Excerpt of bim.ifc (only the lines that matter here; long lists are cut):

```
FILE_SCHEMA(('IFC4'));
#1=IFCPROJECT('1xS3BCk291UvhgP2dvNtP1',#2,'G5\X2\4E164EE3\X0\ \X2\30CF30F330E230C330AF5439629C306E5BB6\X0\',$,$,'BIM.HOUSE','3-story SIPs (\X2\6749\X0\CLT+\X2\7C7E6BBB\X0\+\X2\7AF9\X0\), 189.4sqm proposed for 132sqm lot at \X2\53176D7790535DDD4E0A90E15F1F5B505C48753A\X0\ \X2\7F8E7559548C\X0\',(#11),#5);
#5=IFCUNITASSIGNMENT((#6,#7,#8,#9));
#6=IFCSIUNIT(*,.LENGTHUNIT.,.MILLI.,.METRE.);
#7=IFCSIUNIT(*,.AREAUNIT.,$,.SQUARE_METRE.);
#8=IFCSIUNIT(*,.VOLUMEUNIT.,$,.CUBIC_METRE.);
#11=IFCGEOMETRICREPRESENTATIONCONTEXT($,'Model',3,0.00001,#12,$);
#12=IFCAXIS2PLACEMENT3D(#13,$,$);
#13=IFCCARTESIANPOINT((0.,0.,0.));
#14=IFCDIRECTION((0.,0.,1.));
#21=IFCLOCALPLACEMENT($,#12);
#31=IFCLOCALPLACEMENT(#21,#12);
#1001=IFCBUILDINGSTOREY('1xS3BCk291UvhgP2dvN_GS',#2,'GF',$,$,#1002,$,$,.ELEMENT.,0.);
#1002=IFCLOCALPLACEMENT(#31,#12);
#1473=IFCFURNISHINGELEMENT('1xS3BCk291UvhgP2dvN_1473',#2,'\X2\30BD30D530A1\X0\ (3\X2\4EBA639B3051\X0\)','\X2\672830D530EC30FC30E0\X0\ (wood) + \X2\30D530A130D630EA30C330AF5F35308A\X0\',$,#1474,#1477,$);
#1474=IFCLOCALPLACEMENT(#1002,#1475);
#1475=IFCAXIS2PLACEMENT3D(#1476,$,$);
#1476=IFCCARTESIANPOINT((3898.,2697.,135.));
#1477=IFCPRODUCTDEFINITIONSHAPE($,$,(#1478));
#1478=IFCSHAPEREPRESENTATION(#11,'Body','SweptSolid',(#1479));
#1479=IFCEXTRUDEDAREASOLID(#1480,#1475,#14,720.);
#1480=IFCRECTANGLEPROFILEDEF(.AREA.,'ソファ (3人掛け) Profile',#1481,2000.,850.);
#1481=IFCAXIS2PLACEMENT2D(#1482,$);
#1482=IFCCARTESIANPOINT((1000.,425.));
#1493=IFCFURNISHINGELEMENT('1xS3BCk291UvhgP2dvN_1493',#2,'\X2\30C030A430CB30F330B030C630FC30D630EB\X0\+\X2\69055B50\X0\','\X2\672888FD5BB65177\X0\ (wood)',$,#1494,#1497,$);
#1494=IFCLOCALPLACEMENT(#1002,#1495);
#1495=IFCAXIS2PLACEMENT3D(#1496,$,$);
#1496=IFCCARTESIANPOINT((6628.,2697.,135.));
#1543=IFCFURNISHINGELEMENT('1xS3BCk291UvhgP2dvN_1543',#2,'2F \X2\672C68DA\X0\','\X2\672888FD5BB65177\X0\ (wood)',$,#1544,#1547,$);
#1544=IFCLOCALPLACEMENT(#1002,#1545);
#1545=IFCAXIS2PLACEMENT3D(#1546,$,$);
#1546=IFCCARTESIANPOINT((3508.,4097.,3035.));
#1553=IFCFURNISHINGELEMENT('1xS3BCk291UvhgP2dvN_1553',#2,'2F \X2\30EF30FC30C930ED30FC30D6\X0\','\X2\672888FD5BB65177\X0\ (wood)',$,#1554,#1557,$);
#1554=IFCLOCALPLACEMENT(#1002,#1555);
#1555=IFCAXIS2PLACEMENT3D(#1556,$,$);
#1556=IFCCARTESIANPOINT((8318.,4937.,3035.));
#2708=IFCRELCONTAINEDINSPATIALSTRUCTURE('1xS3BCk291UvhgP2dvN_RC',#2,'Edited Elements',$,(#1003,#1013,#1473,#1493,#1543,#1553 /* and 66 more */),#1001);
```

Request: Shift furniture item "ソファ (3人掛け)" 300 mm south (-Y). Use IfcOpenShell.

```python
import ifcopenshell
import ifcopenshell.api.geometry
import ifcopenshell.util.placement

model = ifcopenshell.open("bim.ifc")

item = model.by_guid("1xS3BCk291UvhgP2dvN_1473")
matrix = ifcopenshell.util.placement.get_local_placement(item.ObjectPlacement)
matrix[1, 3] -= 300.0
ifcopenshell.api.geometry.edit_object_placement(model, product=item, matrix=matrix, is_si=False)

print(ifcopenshell.util.placement.get_local_placement(item.ObjectPlacement).round(3) + 0.0)

model.write("bim_rev.ifc")
```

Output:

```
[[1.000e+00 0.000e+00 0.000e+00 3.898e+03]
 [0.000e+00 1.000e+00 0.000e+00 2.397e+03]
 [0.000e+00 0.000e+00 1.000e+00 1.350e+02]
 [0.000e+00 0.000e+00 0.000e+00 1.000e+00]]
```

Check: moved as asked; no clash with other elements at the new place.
